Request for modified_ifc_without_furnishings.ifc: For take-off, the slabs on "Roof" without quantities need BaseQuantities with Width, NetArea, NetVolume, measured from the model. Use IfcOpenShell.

First a look at what the model holds.

```python
import ifcopenshell
import ifcopenshell.util.element
import ifcopenshell.util.unit

model = ifcopenshell.open("modified_ifc_without_furnishings.ifc")
print(model.schema)
for unit_type in ("LENGTHUNIT", "AREAUNIT", "VOLUMEUNIT"):
    print(unit_type, ifcopenshell.util.unit.calculate_unit_scale(model, unit_type))
storey = next(s for s in model.by_type("IfcBuildingStorey") if s.Name == "Roof")
slabs = [e for e in ifcopenshell.util.element.get_decomposition(storey) if e.is_a("IfcSlab")]
for e in sorted(slabs, key=lambda e: e.id()):
    print(e.id(), e.is_a(), e.Name, list(ifcopenshell.util.element.get_psets(e, qtos_only=True)), sep=" | ")
```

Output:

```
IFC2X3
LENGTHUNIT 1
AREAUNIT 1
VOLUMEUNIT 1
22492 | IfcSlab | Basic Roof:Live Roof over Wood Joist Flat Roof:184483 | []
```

```python
import ifcopenshell
import ifcopenshell.api.pset
import ifcopenshell.geom
import ifcopenshell.util.element
import ifcopenshell.util.shape
import ifcopenshell.util.unit

model = ifcopenshell.open("modified_ifc_without_furnishings.ifc")
unit_scale = ifcopenshell.util.unit.calculate_unit_scale(model)
area_scale = ifcopenshell.util.unit.calculate_unit_scale(model, "AREAUNIT")
volume_scale = ifcopenshell.util.unit.calculate_unit_scale(model, "VOLUMEUNIT")
settings = ifcopenshell.geom.settings()

storey = next(s for s in model.by_type("IfcBuildingStorey") if s.Name == "Roof")
slabs = [e for e in ifcopenshell.util.element.get_decomposition(storey) if e.is_a("IfcSlab")]

for e in sorted(slabs, key=lambda e: e.id()):
    if ifcopenshell.util.element.get_psets(e, qtos_only=True, should_inherit=False):
        continue
    # Geometry comes back in metres, in the element's own axes.
    shape = ifcopenshell.geom.create_shape(settings, e)
    values = {
        "Width": ifcopenshell.util.shape.get_z(shape.geometry) / unit_scale,
        "NetArea": ifcopenshell.util.shape.get_footprint_area(shape.geometry) / area_scale,
        "NetVolume": ifcopenshell.util.shape.get_volume(shape.geometry) / volume_scale,
    }
    qto = ifcopenshell.api.pset.add_qto(model, product=e, name="BaseQuantities")
    ifcopenshell.api.pset.edit_qto(model, qto=qto, properties=values)
    print(e.id(), {k: round(v, 3) for k, v in values.items()})

model.write("modified_ifc_without_furnishings_edited.ifc")
```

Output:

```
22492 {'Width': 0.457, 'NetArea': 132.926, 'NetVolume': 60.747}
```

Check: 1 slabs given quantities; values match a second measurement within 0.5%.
